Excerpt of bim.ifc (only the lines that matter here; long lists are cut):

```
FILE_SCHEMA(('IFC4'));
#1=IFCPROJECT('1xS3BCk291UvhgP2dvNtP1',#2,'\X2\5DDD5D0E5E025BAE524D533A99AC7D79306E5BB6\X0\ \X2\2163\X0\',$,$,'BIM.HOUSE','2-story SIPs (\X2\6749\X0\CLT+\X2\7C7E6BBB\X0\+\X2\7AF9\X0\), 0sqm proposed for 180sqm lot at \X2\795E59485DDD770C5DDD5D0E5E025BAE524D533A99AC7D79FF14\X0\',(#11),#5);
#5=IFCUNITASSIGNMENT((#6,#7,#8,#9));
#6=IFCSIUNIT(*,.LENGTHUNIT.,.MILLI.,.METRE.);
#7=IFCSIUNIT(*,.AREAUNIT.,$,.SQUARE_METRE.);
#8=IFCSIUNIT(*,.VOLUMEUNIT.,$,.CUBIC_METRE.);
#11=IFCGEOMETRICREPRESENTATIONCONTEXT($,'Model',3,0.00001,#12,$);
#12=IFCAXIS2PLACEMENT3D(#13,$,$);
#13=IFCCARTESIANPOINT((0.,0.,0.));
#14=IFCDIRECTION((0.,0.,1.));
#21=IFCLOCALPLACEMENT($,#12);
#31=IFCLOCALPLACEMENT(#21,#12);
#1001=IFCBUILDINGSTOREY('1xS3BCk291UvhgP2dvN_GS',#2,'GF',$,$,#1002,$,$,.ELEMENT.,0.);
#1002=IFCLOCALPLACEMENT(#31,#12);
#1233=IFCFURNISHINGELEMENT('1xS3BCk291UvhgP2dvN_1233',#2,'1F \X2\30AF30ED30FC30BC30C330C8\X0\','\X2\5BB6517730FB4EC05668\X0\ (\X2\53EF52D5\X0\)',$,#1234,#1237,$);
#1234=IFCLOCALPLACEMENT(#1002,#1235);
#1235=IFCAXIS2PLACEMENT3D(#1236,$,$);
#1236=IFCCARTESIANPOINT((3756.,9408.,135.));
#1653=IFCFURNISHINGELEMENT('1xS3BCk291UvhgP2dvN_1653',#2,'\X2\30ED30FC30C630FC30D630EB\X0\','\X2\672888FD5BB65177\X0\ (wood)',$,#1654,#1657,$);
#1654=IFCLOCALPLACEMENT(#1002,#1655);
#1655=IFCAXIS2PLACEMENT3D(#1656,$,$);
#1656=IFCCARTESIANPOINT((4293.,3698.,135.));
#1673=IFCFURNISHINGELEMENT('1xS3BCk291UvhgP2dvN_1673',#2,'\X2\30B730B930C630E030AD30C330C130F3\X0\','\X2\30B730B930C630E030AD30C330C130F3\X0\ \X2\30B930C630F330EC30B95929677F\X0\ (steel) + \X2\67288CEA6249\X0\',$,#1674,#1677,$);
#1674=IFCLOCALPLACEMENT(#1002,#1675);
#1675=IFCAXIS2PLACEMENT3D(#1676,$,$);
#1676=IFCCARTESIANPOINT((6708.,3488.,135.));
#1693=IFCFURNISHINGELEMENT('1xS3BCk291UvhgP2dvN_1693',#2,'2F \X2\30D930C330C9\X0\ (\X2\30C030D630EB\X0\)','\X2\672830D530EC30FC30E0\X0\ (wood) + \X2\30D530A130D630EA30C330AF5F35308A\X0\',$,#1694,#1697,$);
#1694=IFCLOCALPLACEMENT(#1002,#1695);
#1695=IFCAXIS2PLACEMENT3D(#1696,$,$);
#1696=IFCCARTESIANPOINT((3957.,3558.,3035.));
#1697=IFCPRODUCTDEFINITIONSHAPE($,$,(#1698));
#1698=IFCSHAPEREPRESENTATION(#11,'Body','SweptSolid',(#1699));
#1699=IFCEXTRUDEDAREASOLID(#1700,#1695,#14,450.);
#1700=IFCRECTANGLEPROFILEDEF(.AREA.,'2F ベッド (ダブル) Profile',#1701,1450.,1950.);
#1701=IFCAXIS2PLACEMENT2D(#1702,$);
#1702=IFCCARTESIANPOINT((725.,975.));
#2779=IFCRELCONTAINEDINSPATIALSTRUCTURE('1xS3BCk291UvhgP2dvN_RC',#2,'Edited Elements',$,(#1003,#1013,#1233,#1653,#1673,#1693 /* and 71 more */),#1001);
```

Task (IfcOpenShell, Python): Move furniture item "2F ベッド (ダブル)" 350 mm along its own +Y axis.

```python
import ifcopenshell
import ifcopenshell.api.geometry
import ifcopenshell.util.placement

model = ifcopenshell.open("bim.ifc")

item = model.by_guid("1xS3BCk291UvhgP2dvN_1693")
matrix = ifcopenshell.util.placement.get_local_placement(item.ObjectPlacement)
matrix[:3, 3] += matrix[:3, 1] * 350.0
ifcopenshell.api.geometry.edit_object_placement(model, product=item, matrix=matrix, is_si=False)

print(ifcopenshell.util.placement.get_local_placement(item.ObjectPlacement).round(3) + 0.0)

model.write("bim_updated.ifc")
```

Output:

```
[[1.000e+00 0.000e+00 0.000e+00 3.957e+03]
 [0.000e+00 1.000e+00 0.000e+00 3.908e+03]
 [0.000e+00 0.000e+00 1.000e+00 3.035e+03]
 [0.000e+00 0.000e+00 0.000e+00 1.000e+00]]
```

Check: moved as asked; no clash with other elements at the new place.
